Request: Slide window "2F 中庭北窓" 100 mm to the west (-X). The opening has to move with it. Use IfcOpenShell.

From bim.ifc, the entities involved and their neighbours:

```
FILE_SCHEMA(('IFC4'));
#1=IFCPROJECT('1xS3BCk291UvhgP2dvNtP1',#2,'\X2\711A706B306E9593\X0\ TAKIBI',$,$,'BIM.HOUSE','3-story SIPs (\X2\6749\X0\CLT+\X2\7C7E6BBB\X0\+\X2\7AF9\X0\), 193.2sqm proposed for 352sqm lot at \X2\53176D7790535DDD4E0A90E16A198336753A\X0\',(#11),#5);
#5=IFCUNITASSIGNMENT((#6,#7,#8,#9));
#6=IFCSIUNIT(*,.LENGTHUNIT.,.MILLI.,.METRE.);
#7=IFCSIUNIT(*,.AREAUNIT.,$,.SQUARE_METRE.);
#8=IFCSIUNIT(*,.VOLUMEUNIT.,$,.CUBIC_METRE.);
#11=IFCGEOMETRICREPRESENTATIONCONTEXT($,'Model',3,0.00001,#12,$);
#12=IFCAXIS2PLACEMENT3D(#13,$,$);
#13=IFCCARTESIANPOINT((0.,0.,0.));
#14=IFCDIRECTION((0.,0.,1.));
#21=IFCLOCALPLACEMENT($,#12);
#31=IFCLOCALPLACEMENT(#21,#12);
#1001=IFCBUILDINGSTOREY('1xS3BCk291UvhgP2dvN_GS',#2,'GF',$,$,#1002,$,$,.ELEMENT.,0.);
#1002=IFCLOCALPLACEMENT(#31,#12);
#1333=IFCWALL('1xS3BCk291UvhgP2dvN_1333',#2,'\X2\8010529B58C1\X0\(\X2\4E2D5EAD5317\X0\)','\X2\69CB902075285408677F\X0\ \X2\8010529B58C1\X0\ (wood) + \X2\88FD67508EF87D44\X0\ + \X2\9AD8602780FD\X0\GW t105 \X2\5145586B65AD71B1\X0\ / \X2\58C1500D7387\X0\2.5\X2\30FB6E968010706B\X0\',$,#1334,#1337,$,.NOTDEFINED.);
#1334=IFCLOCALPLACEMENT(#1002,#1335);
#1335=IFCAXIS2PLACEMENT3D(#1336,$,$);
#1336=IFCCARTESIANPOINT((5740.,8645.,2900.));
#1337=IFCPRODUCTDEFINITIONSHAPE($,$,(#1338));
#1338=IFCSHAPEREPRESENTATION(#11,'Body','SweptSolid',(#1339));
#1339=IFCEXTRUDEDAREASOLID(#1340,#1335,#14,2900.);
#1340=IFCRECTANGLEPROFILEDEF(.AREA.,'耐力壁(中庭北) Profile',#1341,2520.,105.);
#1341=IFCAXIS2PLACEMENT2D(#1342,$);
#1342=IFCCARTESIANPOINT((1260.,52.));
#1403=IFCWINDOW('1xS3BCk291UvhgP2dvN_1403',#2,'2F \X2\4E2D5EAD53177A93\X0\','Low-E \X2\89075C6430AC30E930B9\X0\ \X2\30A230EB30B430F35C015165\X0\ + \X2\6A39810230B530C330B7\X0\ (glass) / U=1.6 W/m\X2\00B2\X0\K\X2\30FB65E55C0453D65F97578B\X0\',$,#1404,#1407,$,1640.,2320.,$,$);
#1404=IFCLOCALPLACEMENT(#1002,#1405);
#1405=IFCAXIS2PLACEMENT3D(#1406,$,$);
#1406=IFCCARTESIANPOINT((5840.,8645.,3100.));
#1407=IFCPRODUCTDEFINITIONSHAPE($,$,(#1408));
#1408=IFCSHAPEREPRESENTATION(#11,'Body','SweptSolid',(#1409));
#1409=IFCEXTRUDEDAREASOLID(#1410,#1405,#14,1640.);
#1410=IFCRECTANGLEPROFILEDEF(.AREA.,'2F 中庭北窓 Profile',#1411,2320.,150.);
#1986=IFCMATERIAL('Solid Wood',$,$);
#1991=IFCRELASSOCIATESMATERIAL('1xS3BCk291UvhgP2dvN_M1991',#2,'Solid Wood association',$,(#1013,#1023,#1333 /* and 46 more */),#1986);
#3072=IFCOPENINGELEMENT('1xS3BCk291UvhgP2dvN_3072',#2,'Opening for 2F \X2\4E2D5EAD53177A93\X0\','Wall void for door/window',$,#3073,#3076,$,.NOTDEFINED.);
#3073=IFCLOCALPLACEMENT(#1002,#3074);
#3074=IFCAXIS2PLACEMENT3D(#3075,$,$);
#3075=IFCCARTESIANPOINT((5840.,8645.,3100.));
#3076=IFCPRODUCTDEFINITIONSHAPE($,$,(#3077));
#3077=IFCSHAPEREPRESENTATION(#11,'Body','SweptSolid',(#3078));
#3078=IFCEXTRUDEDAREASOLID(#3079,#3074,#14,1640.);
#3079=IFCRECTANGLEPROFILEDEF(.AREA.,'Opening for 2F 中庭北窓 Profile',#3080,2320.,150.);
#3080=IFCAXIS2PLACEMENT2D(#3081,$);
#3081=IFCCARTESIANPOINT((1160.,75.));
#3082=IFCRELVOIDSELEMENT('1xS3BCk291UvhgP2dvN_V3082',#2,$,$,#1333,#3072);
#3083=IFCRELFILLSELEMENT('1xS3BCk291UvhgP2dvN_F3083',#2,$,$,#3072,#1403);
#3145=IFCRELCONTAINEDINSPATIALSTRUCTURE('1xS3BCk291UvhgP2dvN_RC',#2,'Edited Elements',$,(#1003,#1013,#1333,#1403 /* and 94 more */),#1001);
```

```python
import ifcopenshell
import ifcopenshell.api.geometry
import ifcopenshell.util.placement
import ifcopenshell.util.unit

model = ifcopenshell.open("bim.ifc")
unit_scale = ifcopenshell.util.unit.calculate_unit_scale(model)

window = model.by_guid("1xS3BCk291UvhgP2dvN_1403")
opening = window.FillsVoids[0].RelatingOpeningElement
wall = opening.VoidsElements[0].RelatingBuildingElement

wall_matrix = ifcopenshell.util.placement.get_local_placement(wall.ObjectPlacement)
shift = wall_matrix[:3, 0] * -0.1 / unit_scale
before = ifcopenshell.util.placement.get_local_placement(window.ObjectPlacement)[:3, 3].copy()

# The window is not placed relative to its opening, so move both.
for product in (opening, window):
    matrix = ifcopenshell.util.placement.get_local_placement(product.ObjectPlacement)
    matrix[:3, 3] += shift
    ifcopenshell.api.geometry.edit_object_placement(model, product=product, matrix=matrix, is_si=False)

after = ifcopenshell.util.placement.get_local_placement(window.ObjectPlacement)[:3, 3]
print("window moved by", (after - before).round(3) + 0.0)

model.write("bim_updated.ifc")
```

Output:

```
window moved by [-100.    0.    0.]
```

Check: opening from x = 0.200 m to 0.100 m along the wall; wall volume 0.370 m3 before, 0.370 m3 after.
